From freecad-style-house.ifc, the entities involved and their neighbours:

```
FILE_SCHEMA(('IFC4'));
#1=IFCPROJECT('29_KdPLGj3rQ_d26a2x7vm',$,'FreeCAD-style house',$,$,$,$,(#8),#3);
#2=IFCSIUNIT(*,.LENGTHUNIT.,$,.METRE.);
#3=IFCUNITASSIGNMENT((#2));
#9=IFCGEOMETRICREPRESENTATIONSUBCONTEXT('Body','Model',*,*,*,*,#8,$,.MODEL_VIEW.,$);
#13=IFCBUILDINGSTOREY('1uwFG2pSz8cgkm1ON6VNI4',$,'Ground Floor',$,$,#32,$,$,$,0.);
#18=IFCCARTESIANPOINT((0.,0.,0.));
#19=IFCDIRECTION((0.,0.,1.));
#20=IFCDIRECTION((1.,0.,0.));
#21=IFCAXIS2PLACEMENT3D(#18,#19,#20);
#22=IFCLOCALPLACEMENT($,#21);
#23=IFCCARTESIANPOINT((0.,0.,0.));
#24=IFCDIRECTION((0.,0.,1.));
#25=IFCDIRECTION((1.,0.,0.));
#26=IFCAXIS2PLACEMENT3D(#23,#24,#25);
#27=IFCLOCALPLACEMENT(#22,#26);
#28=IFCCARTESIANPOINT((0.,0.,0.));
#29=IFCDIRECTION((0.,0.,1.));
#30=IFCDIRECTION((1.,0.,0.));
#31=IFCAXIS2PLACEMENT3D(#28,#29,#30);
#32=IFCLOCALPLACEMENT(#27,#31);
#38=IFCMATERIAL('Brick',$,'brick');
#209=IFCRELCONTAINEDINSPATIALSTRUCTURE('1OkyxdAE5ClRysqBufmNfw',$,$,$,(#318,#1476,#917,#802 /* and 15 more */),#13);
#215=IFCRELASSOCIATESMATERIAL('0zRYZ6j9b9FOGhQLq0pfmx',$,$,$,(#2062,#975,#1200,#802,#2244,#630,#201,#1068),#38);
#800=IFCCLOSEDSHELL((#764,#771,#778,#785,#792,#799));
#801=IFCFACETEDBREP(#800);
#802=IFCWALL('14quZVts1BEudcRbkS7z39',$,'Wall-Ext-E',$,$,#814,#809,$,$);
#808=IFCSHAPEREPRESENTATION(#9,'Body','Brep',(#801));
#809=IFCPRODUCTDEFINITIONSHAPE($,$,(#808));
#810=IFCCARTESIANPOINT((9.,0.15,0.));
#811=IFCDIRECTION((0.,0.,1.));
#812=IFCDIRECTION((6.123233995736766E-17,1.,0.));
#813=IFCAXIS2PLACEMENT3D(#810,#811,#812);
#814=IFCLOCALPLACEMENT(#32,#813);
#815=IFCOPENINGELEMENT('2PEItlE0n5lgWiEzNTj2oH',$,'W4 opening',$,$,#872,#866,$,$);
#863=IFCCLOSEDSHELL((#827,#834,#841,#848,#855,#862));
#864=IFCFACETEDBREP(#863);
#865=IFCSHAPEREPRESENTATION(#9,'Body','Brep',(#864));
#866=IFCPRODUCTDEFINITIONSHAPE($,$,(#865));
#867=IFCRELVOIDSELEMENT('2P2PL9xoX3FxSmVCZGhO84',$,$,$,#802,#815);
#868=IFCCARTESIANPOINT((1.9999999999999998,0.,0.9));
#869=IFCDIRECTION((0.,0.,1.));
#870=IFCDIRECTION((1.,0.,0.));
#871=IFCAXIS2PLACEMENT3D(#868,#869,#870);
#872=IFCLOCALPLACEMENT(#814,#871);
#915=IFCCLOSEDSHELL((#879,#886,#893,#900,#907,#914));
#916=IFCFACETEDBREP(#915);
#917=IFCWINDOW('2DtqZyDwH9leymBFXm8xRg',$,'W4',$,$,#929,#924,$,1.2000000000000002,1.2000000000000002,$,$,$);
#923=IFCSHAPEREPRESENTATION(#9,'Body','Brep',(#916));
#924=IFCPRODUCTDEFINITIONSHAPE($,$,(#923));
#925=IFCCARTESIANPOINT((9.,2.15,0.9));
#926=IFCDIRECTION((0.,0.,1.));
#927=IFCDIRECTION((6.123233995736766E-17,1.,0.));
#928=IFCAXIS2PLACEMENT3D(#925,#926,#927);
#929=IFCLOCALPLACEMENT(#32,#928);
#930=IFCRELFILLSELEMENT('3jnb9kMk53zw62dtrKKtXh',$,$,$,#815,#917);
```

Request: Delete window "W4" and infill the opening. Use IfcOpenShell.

```python
import ifcopenshell
import ifcopenshell.api.feature
import ifcopenshell.api.root
import ifcopenshell.geom
import ifcopenshell.util.shape

model = ifcopenshell.open("freecad-style-house.ifc")
settings = ifcopenshell.geom.settings()


def volume(element):
    """Net volume in cubic metres, openings subtracted."""
    shape = ifcopenshell.geom.create_shape(settings, element)
    return ifcopenshell.util.shape.get_volume(shape.geometry)


window = model.by_guid("2DtqZyDwH9leymBFXm8xRg")
opening = window.FillsVoids[0].RelatingOpeningElement
wall = opening.VoidsElements[0].RelatingBuildingElement
before = volume(wall)

ifcopenshell.api.root.remove_product(model, product=window)
ifcopenshell.api.feature.remove_feature(model, feature=opening)

after = volume(wall)

print(f"wall volume {before:.3f} -> {after:.3f} m3")

model.write("freecad-style-house_rev.ifc")
```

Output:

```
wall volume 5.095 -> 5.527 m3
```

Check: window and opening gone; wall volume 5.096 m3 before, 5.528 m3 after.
